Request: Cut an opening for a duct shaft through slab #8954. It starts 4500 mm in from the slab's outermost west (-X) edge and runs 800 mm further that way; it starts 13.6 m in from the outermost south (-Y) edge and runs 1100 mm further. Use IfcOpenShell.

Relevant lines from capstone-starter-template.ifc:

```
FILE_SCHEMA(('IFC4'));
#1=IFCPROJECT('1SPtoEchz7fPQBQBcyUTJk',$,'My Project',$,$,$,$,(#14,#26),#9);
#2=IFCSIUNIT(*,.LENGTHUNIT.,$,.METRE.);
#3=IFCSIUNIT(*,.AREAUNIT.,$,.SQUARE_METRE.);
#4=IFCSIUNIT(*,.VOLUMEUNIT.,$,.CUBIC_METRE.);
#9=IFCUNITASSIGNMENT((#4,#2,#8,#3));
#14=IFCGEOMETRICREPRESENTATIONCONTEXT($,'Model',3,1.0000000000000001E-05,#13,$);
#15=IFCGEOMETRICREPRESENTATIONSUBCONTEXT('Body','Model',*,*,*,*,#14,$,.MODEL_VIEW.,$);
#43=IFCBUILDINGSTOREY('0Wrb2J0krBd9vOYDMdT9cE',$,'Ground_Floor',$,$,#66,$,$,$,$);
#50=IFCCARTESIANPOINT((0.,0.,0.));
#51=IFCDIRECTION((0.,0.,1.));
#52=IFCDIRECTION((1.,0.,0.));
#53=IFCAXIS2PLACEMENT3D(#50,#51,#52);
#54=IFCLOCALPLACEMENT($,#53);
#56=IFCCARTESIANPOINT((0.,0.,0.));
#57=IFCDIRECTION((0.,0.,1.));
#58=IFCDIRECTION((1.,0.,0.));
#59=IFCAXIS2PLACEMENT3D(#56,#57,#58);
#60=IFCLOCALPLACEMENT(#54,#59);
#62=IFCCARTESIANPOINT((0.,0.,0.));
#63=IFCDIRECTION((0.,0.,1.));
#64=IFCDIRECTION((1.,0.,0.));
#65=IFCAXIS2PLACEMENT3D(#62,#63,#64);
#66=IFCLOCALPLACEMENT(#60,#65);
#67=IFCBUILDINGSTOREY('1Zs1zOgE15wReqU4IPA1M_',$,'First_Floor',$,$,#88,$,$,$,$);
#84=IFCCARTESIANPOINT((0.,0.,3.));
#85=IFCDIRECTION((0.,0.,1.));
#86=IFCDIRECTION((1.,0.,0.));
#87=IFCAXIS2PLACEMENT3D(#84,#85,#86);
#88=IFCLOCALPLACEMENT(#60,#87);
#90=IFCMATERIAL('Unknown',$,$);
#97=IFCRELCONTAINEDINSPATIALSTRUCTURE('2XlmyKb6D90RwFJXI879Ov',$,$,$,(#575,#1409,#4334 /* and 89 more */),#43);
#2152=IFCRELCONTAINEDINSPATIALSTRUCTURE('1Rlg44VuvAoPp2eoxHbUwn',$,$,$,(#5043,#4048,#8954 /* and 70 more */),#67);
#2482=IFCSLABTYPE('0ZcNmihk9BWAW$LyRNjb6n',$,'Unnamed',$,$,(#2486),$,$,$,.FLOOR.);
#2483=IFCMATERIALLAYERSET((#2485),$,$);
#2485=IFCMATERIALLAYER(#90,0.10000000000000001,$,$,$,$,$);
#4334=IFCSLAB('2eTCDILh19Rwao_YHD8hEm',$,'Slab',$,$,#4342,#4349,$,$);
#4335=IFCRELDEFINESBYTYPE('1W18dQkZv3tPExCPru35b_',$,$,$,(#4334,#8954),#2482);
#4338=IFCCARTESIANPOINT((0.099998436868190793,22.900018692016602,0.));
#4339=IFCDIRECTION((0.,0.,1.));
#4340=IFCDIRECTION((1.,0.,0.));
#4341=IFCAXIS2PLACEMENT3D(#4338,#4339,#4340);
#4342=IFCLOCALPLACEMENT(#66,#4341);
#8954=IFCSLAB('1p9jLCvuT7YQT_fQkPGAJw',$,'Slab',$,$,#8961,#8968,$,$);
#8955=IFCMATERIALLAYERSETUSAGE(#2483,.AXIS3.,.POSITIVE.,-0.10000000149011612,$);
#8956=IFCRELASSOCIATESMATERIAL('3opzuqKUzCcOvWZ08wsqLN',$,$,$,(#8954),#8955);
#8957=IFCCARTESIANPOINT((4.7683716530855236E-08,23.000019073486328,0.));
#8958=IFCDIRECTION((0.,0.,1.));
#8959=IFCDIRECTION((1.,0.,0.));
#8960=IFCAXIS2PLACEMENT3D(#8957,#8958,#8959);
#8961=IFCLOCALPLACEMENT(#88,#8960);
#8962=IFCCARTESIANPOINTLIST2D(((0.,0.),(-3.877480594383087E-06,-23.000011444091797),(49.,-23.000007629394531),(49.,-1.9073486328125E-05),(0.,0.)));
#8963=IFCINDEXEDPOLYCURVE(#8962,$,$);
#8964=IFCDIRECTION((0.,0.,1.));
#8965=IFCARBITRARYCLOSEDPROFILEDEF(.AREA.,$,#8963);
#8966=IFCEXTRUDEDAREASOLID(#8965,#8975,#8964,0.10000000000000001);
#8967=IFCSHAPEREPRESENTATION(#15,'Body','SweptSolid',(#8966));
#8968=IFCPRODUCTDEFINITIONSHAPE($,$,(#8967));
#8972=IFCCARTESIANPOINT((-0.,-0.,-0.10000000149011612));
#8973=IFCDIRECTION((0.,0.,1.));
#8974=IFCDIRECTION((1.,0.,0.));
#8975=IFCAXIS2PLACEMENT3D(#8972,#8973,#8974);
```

```python
import numpy as np
import ifcopenshell
import ifcopenshell.api.feature
import ifcopenshell.api.geometry
import ifcopenshell.api.root
import ifcopenshell.geom
import ifcopenshell.util.placement
import ifcopenshell.util.representation
import ifcopenshell.util.shape
import ifcopenshell.util.unit

model = ifcopenshell.open("capstone-starter-template.ifc")
unit_scale = ifcopenshell.util.unit.calculate_unit_scale(model)
settings = ifcopenshell.geom.settings()


def volume(element):
    """Net volume in cubic metres, openings subtracted."""
    shape = ifcopenshell.geom.create_shape(settings, element)
    return ifcopenshell.util.shape.get_volume(shape.geometry)


slab = model.by_guid("1p9jLCvuT7YQT_fQkPGAJw")
before = volume(slab)

# Extent in the slab's own axes, in metres. The edges named are its -X and -Y sides.
slab_shape = ifcopenshell.geom.create_shape(settings, slab)
vertices = ifcopenshell.util.shape.get_vertices(slab_shape.geometry)
x_min, y_min, bottom = vertices.min(axis=0)
top = vertices[:, 2].max()

opening = ifcopenshell.api.root.create_entity(model, ifc_class="IfcOpeningElement", name="Duct shaft opening", predefined_type="OPENING")
context = ifcopenshell.util.representation.get_context(model, "Model", "Body", "MODEL_VIEW")
width, depth = 0.8, 1.1
outline = [(0.0, 0.0), (width, 0.0), (width, depth), (0.0, depth), (0.0, 0.0)]
# Overshoot both faces by 50 mm so the cut is clean.
shape = ifcopenshell.api.geometry.add_slab_representation(
    model, context=context, depth=top - bottom + 0.1, polyline=outline
)
ifcopenshell.api.geometry.assign_representation(model, product=opening, representation=shape)

matrix = ifcopenshell.util.placement.get_local_placement(slab.ObjectPlacement)
matrix[:, 3] = matrix @ np.append(np.array([x_min + 4.5, y_min + 13.6, bottom - 0.05]) / unit_scale, 1.0)
ifcopenshell.api.geometry.edit_object_placement(model, product=opening, matrix=matrix, is_si=False)
ifcopenshell.api.feature.add_feature(model, feature=opening, element=slab)

after = volume(slab)

print(f"slab volume {before:.3f} -> {after:.3f} m3")

model.write("capstone-starter-template_edited.ifc")
```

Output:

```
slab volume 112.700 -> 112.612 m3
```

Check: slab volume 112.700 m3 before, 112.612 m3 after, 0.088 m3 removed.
